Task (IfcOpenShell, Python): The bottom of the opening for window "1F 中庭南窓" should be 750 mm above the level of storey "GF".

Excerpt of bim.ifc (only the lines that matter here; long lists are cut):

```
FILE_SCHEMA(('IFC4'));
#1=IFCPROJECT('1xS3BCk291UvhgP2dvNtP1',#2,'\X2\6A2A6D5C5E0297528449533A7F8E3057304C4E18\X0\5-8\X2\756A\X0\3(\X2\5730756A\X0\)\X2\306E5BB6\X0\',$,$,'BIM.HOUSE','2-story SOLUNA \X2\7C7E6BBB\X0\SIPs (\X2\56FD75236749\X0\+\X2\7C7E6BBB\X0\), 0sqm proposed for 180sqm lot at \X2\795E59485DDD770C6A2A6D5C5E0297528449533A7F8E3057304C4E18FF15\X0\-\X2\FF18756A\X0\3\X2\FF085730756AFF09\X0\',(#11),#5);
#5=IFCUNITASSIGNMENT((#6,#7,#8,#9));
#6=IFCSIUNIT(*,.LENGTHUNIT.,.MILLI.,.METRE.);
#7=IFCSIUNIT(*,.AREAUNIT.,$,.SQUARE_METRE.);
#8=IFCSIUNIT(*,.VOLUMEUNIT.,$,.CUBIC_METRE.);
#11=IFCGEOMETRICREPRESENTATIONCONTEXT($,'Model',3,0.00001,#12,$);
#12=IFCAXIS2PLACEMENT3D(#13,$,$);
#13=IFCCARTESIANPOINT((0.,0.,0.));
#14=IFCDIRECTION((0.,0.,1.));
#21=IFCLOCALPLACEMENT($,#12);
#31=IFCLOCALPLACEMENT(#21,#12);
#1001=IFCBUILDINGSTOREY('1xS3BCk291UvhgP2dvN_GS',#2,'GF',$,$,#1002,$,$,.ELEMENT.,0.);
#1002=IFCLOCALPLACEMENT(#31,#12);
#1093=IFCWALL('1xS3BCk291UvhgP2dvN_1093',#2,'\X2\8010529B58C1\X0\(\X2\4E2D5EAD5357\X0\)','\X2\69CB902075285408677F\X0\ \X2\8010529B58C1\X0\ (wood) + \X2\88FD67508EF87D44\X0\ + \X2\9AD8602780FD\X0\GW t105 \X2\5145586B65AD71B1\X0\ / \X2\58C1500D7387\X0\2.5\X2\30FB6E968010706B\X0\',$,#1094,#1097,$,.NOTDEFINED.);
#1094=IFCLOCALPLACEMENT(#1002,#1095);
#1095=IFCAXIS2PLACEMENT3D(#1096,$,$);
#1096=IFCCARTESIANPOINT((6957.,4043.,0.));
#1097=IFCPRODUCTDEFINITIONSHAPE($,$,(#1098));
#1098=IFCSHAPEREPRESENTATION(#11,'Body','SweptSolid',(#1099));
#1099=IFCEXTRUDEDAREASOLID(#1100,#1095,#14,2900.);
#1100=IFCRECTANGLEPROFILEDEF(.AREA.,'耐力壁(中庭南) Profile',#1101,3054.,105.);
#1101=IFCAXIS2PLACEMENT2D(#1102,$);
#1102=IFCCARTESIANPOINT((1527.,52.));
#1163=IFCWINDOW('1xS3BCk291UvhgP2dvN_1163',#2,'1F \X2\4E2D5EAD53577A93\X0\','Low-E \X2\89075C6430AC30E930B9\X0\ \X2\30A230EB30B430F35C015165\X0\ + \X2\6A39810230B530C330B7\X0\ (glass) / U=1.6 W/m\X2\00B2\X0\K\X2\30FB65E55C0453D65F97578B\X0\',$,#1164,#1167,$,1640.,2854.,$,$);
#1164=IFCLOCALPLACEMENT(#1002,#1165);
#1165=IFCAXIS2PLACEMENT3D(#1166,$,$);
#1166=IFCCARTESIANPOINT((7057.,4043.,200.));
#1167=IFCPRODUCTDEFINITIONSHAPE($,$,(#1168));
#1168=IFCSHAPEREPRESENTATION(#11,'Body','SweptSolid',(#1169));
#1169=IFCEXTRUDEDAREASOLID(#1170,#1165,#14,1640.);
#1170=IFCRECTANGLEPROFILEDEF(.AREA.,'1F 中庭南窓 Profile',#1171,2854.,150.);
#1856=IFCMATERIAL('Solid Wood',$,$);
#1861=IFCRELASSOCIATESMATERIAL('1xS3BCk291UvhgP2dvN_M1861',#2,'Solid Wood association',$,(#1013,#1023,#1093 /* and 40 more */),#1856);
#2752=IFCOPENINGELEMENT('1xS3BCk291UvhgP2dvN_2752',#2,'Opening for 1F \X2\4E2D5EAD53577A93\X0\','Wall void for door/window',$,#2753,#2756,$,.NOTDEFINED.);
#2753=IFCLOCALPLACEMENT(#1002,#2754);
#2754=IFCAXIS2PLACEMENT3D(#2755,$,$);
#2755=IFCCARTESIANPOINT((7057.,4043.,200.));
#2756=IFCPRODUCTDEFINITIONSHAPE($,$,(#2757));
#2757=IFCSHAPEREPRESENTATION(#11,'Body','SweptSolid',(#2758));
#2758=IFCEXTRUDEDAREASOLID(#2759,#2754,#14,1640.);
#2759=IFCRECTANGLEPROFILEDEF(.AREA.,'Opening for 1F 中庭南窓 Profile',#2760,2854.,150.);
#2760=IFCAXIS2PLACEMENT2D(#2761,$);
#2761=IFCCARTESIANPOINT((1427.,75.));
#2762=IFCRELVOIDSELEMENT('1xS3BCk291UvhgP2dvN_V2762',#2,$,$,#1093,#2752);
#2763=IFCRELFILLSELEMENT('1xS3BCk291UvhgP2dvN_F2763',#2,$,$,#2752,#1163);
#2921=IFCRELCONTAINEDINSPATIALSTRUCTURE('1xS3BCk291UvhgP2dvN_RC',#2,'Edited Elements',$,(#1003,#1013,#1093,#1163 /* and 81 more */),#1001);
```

```python
import numpy as np
import ifcopenshell
import ifcopenshell.api.geometry
import ifcopenshell.geom
import ifcopenshell.util.element
import ifcopenshell.util.placement
import ifcopenshell.util.shape
import ifcopenshell.util.unit

model = ifcopenshell.open("bim.ifc")
unit_scale = ifcopenshell.util.unit.calculate_unit_scale(model)

window = model.by_guid("1xS3BCk291UvhgP2dvN_1163")
opening = window.FillsVoids[0].RelatingOpeningElement
storey = ifcopenshell.util.element.get_container(window, ifc_class="IfcBuildingStorey")
level = ifcopenshell.util.placement.get_local_placement(storey.ObjectPlacement)[2, 3]

# The opening's origin need not be at the sill, so measure its lowest point.
shape = ifcopenshell.geom.create_shape(ifcopenshell.geom.settings(), opening)
bottom = ifcopenshell.util.shape.get_shape_bottom_elevation(shape, shape.geometry) / unit_scale
dz = level + 750.0 - bottom

shift = np.array([0.0, 0.0, dz])
# The window is not placed relative to its opening, so move both.
for product in (opening, window):
    matrix = ifcopenshell.util.placement.get_local_placement(product.ObjectPlacement)
    matrix[:3, 3] += shift
    ifcopenshell.api.geometry.edit_object_placement(model, product=product, matrix=matrix, is_si=False)

print(f"moved by {dz * unit_scale:+.3f} m")

model.write("bim_v2.ifc")
```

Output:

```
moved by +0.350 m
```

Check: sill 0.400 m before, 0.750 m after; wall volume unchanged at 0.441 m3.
